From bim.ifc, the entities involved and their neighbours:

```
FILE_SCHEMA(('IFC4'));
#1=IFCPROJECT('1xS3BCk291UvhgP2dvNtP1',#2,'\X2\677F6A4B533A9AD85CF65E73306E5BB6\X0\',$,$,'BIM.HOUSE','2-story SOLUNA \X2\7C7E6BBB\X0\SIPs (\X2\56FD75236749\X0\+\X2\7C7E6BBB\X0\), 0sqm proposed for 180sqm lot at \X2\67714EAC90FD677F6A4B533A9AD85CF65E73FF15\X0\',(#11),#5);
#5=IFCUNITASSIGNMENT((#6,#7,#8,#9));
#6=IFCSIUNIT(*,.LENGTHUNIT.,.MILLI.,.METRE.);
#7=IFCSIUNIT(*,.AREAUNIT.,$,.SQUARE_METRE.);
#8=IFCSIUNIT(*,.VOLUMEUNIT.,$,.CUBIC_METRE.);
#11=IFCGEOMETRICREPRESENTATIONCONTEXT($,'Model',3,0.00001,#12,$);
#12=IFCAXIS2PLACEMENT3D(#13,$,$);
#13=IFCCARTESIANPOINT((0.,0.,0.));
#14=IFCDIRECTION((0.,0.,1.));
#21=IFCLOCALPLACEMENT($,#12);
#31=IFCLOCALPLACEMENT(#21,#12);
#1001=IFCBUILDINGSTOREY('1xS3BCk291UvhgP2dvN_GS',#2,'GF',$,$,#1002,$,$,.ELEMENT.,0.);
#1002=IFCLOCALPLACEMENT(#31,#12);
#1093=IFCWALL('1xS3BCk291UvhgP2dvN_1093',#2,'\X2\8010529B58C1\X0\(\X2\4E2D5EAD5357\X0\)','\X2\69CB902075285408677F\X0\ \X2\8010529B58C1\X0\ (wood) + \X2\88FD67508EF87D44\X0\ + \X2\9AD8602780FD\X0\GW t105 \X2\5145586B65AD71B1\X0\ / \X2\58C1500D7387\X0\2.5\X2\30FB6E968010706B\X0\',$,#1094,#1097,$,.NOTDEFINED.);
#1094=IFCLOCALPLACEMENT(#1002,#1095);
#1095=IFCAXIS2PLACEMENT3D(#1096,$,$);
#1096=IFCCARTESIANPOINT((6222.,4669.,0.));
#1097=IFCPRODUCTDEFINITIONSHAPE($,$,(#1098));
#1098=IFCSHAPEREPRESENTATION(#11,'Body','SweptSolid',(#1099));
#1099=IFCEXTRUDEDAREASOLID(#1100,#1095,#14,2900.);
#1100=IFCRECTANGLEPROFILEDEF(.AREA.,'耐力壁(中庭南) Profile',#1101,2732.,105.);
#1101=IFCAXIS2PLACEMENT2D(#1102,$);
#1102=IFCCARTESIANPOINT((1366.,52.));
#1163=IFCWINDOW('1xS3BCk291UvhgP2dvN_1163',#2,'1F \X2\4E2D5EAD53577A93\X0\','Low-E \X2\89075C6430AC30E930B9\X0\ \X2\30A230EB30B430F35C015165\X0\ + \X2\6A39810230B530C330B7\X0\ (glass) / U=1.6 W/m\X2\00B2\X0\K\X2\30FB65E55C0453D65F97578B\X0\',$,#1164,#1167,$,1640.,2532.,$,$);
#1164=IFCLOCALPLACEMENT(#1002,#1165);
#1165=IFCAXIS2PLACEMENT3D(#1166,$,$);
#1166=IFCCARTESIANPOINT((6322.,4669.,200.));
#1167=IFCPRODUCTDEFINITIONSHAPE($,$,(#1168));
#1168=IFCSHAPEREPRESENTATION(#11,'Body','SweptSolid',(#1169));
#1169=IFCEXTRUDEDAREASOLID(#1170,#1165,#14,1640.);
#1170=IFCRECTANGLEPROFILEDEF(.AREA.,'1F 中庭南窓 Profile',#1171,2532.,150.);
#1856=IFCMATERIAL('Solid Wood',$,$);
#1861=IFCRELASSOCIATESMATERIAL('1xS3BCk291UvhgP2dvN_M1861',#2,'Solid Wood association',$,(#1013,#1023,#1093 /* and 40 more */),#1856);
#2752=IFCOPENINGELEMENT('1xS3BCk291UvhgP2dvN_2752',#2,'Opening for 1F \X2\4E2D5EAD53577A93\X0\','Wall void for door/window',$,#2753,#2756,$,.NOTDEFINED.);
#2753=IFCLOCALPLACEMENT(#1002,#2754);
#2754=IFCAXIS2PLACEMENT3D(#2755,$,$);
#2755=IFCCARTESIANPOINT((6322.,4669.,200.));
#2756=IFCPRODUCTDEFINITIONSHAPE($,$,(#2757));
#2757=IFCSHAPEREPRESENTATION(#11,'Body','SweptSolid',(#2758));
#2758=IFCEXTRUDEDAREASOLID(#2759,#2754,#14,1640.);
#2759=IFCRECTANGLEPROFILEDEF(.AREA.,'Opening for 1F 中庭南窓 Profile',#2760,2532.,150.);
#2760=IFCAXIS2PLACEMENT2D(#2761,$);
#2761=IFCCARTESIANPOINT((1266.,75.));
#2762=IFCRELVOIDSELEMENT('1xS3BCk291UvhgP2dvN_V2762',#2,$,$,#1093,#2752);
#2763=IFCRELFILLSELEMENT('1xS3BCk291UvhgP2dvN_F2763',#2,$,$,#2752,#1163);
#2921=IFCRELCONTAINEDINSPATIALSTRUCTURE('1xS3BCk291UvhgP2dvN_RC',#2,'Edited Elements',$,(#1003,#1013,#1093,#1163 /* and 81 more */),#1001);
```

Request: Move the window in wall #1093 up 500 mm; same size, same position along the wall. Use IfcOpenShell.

```python
import numpy as np
import ifcopenshell
import ifcopenshell.api.geometry
import ifcopenshell.util.placement
import ifcopenshell.util.unit

model = ifcopenshell.open("bim.ifc")
unit_scale = ifcopenshell.util.unit.calculate_unit_scale(model)

window = model.by_guid("1xS3BCk291UvhgP2dvN_1163")
opening = window.FillsVoids[0].RelatingOpeningElement
dz = 0.5 / unit_scale

shift = np.array([0.0, 0.0, dz])
# The window is not placed relative to its opening, so move both.
for product in (opening, window):
    matrix = ifcopenshell.util.placement.get_local_placement(product.ObjectPlacement)
    matrix[:3, 3] += shift
    ifcopenshell.api.geometry.edit_object_placement(model, product=product, matrix=matrix, is_si=False)

print(f"moved by {dz * unit_scale:+.3f} m")

model.write("bim_updated.ifc")
```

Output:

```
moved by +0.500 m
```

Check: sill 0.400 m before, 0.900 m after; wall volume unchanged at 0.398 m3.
